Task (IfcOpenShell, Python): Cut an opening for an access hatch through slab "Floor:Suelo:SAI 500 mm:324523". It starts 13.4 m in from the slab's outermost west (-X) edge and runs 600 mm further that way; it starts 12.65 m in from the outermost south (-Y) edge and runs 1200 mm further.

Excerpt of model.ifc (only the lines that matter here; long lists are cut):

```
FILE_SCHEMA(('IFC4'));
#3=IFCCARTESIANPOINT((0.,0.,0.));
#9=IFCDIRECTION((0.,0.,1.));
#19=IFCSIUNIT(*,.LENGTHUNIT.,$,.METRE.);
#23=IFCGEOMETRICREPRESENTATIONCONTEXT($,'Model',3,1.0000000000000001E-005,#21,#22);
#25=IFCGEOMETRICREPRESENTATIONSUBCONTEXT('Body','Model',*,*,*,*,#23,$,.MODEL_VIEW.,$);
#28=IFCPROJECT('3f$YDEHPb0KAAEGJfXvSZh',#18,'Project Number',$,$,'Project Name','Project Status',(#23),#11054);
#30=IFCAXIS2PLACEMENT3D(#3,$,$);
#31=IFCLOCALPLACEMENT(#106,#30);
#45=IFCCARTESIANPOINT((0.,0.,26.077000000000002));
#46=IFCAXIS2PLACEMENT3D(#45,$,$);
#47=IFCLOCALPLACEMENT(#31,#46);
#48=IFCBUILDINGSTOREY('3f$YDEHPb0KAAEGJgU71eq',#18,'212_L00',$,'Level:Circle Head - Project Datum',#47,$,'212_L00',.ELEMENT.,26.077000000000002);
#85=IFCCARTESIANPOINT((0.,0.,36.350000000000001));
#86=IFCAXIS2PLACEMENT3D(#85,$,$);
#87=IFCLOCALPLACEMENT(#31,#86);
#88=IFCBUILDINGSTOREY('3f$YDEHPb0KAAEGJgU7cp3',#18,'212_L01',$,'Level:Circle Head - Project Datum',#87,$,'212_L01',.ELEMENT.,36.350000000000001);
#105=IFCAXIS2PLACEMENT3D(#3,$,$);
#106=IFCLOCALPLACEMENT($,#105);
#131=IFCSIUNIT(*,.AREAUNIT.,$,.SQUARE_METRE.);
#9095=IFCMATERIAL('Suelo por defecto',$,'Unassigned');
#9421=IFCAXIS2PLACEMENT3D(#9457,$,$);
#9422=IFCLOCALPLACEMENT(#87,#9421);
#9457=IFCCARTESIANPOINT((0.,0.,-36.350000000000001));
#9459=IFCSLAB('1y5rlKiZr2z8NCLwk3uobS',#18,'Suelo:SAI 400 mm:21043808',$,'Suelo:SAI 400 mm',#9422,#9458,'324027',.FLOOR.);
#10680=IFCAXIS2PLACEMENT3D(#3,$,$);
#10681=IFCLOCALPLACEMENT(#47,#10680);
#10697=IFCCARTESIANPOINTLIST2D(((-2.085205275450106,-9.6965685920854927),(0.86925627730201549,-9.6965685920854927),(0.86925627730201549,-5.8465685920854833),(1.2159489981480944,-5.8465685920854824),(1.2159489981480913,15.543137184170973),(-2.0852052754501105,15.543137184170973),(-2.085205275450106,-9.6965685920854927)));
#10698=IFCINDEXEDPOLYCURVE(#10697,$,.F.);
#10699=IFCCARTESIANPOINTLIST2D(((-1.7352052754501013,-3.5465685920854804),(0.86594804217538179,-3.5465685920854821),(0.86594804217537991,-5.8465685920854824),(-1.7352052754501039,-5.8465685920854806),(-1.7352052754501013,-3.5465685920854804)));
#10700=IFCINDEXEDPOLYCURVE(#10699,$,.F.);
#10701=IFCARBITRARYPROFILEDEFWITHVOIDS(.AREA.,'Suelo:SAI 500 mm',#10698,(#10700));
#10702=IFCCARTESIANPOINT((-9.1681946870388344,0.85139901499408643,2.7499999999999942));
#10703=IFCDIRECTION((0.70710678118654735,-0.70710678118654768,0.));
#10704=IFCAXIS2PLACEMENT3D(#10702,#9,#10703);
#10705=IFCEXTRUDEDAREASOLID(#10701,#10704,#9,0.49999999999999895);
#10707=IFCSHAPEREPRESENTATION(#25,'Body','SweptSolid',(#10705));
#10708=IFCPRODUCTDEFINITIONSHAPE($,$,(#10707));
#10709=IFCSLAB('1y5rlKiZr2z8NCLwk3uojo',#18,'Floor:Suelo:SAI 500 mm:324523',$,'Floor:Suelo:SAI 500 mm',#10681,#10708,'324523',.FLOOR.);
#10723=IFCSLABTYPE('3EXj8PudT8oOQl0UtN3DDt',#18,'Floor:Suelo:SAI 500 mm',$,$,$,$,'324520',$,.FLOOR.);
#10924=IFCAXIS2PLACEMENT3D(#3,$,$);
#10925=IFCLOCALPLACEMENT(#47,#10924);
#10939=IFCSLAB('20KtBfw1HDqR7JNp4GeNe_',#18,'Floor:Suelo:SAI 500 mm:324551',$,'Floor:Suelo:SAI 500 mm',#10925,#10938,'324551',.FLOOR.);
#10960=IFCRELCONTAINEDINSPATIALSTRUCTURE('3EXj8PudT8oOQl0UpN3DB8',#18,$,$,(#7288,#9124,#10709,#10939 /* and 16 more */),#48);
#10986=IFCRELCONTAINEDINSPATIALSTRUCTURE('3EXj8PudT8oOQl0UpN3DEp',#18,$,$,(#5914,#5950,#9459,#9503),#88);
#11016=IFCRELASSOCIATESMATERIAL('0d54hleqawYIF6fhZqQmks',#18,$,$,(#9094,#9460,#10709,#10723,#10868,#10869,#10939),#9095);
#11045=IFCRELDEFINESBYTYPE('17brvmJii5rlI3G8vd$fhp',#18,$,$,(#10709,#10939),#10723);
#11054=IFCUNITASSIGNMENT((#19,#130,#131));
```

```python
import numpy as np
import ifcopenshell
import ifcopenshell.api.feature
import ifcopenshell.api.geometry
import ifcopenshell.api.root
import ifcopenshell.geom
import ifcopenshell.util.placement
import ifcopenshell.util.representation
import ifcopenshell.util.shape
import ifcopenshell.util.unit

model = ifcopenshell.open("model.ifc")
unit_scale = ifcopenshell.util.unit.calculate_unit_scale(model)
settings = ifcopenshell.geom.settings()


def volume(element):
    """Net volume in cubic metres, openings subtracted."""
    shape = ifcopenshell.geom.create_shape(settings, element)
    return ifcopenshell.util.shape.get_volume(shape.geometry)


slab = model.by_guid("1y5rlKiZr2z8NCLwk3uojo")
before = volume(slab)

# Extent in the slab's own axes, in metres. The edges named are its -X and -Y sides.
slab_shape = ifcopenshell.geom.create_shape(settings, slab)
vertices = ifcopenshell.util.shape.get_vertices(slab_shape.geometry)
x_min, y_min, bottom = vertices.min(axis=0)
top = vertices[:, 2].max()

opening = ifcopenshell.api.root.create_entity(model, ifc_class="IfcOpeningElement", name="Access hatch opening", predefined_type="OPENING")
context = ifcopenshell.util.representation.get_context(model, "Model", "Body", "MODEL_VIEW")
width, depth = 0.6, 1.2
outline = [(0.0, 0.0), (width, 0.0), (width, depth), (0.0, depth), (0.0, 0.0)]
# Overshoot both faces by 50 mm so the cut is clean.
shape = ifcopenshell.api.geometry.add_slab_representation(
    model, context=context, depth=top - bottom + 0.1, polyline=outline
)
ifcopenshell.api.geometry.assign_representation(model, product=opening, representation=shape)

matrix = ifcopenshell.util.placement.get_local_placement(slab.ObjectPlacement)
matrix[:, 3] = matrix @ np.append(np.array([x_min + 13.4, y_min + 12.65, bottom - 0.05]) / unit_scale, 1.0)
ifcopenshell.api.geometry.edit_object_placement(model, product=opening, matrix=matrix, is_si=False)
ifcopenshell.api.feature.add_feature(model, feature=opening, element=slab)

after = volume(slab)

print(f"slab volume {before:.3f} -> {after:.3f} m3")

model.write("model_updated.ifc")
```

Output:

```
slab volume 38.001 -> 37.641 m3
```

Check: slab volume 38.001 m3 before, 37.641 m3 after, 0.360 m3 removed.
